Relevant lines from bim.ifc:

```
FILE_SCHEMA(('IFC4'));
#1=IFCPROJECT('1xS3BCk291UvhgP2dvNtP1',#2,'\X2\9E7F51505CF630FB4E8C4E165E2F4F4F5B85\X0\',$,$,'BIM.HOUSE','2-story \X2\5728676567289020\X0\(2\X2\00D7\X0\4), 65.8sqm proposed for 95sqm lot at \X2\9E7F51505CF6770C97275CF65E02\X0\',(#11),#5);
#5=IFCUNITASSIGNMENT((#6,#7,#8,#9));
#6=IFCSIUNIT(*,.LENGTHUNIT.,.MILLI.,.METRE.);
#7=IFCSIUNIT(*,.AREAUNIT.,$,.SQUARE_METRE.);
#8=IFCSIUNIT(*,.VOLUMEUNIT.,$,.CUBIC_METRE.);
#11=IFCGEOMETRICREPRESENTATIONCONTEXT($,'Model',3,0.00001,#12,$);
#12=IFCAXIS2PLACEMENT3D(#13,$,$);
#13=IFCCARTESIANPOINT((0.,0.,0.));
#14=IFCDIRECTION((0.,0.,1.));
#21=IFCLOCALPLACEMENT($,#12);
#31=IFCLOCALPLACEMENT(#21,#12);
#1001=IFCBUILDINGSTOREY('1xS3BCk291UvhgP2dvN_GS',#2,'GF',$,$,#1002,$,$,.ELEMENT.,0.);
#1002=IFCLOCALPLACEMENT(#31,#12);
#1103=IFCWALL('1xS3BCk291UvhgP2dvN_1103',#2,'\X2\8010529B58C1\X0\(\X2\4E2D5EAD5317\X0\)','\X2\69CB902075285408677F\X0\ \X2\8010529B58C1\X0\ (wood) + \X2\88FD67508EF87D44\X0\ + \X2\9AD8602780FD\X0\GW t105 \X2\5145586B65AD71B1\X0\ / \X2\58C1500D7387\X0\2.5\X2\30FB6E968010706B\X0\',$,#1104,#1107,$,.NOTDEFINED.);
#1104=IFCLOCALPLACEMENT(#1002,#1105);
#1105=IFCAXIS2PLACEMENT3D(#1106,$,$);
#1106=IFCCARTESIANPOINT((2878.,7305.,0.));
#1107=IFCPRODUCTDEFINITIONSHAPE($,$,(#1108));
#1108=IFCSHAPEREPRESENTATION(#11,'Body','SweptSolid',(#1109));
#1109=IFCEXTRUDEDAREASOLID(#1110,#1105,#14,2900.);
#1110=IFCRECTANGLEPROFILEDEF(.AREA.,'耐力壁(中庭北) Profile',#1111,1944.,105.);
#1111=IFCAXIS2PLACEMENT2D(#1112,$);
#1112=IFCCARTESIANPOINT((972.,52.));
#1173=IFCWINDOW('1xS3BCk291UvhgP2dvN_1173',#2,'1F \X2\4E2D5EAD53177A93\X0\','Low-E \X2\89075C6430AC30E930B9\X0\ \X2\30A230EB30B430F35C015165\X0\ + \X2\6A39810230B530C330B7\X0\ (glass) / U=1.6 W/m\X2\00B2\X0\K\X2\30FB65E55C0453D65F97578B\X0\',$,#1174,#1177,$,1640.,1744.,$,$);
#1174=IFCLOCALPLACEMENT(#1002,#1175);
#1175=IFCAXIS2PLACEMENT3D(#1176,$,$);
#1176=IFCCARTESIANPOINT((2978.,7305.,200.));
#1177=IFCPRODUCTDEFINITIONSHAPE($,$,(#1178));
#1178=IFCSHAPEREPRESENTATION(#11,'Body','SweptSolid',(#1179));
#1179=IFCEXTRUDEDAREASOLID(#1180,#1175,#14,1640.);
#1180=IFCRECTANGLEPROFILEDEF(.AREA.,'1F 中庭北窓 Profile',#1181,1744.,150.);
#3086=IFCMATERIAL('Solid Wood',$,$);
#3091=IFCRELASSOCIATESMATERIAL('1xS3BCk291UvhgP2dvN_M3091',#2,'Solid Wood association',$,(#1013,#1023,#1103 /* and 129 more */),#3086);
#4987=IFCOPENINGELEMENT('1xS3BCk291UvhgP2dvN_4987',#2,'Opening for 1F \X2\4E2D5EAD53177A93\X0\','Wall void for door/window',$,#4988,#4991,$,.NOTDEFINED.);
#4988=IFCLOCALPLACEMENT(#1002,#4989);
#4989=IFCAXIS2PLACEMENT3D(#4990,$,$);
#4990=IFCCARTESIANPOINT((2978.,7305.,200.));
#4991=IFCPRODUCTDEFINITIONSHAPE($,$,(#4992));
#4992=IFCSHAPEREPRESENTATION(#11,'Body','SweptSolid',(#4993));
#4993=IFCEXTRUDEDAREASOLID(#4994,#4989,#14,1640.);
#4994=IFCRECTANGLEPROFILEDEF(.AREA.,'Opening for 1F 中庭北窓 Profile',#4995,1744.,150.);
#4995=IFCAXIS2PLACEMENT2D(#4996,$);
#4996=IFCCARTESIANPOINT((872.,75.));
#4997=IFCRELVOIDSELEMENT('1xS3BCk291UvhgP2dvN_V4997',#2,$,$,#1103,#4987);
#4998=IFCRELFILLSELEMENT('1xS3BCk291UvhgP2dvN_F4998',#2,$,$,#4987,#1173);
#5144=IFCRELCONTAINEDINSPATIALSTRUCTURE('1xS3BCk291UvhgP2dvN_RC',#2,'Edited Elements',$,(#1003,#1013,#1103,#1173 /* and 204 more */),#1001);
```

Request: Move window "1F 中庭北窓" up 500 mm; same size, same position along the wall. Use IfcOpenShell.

```python
import numpy as np
import ifcopenshell
import ifcopenshell.api.geometry
import ifcopenshell.util.placement
import ifcopenshell.util.unit

model = ifcopenshell.open("bim.ifc")
unit_scale = ifcopenshell.util.unit.calculate_unit_scale(model)

window = model.by_guid("1xS3BCk291UvhgP2dvN_1173")
opening = window.FillsVoids[0].RelatingOpeningElement
dz = 0.5 / unit_scale

shift = np.array([0.0, 0.0, dz])
# The window is not placed relative to its opening, so move both.
for product in (opening, window):
    matrix = ifcopenshell.util.placement.get_local_placement(product.ObjectPlacement)
    matrix[:3, 3] += shift
    ifcopenshell.api.geometry.edit_object_placement(model, product=product, matrix=matrix, is_si=False)

print(f"moved by {dz * unit_scale:+.3f} m")

model.write("bim_rev.ifc")
```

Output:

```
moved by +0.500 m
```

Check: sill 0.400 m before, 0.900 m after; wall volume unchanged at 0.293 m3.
